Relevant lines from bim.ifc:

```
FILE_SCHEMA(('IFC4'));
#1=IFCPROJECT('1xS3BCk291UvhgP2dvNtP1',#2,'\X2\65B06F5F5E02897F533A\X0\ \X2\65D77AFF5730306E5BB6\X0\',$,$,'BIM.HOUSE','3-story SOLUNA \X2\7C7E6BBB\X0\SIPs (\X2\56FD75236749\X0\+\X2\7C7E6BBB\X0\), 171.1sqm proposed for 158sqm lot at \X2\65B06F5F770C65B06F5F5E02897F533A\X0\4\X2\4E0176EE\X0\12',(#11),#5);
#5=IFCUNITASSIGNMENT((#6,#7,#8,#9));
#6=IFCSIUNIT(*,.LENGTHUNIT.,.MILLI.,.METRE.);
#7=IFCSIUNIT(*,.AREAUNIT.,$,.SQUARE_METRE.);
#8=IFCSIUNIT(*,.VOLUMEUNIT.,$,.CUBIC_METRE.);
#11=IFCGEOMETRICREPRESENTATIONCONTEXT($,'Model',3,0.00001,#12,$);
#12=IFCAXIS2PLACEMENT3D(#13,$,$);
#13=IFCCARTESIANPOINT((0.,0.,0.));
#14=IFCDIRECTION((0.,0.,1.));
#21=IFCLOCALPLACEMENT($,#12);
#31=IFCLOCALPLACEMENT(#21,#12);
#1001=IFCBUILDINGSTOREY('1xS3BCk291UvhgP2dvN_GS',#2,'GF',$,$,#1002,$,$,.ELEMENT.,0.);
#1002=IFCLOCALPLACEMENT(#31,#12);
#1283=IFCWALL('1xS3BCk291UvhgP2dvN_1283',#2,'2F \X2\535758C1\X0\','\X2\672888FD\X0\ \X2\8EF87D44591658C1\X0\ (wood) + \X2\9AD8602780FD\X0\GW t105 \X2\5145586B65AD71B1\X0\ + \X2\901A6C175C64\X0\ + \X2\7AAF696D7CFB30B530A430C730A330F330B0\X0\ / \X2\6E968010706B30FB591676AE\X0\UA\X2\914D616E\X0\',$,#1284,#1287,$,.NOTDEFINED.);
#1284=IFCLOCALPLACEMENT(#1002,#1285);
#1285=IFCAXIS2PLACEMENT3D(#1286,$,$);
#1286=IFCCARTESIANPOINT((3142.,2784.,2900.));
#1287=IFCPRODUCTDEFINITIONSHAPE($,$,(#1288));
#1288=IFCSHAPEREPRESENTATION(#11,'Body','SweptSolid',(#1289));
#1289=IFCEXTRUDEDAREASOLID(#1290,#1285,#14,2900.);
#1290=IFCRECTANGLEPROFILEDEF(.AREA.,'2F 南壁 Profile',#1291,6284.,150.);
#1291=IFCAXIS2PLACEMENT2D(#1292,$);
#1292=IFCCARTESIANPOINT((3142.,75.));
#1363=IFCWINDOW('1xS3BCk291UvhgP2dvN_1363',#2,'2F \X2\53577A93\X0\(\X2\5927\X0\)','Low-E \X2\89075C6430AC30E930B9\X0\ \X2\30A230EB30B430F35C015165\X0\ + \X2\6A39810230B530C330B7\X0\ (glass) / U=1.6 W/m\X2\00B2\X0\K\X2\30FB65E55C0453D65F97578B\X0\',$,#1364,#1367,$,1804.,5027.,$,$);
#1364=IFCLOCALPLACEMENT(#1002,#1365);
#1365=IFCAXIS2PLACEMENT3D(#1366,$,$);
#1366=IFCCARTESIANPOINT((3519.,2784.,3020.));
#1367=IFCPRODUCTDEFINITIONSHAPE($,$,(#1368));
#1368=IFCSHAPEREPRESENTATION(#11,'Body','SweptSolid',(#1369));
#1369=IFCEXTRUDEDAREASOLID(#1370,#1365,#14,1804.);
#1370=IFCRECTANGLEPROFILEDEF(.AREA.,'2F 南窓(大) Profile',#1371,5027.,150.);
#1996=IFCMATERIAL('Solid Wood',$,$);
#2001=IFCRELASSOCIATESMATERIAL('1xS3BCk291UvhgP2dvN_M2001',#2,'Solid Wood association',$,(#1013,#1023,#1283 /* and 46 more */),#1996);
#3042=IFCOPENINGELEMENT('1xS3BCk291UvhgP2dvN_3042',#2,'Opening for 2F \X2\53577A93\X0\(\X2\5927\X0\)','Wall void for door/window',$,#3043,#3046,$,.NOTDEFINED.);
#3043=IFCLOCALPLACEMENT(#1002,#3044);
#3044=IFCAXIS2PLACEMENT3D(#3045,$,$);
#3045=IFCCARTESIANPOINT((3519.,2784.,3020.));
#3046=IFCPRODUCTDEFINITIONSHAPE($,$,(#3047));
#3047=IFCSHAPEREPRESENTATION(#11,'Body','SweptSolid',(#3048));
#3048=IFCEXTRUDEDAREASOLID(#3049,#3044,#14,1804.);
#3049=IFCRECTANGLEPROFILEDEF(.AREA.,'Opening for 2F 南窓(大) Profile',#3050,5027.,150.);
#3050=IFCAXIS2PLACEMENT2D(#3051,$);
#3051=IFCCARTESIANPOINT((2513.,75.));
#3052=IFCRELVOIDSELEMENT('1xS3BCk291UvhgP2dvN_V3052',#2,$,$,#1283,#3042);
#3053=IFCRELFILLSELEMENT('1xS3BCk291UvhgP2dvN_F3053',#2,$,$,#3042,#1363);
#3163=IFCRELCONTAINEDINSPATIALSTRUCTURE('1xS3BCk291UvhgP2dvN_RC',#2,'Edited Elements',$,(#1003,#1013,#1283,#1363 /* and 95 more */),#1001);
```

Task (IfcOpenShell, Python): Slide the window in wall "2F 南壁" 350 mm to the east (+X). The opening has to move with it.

```python
import ifcopenshell
import ifcopenshell.api.geometry
import ifcopenshell.util.placement

model = ifcopenshell.open("bim.ifc")

window = model.by_guid("1xS3BCk291UvhgP2dvN_1363")
opening = window.FillsVoids[0].RelatingOpeningElement
wall = opening.VoidsElements[0].RelatingBuildingElement

wall_matrix = ifcopenshell.util.placement.get_local_placement(wall.ObjectPlacement)
shift = wall_matrix[:3, 0] * 350.0
before = ifcopenshell.util.placement.get_local_placement(window.ObjectPlacement)[:3, 3].copy()

# The window is not placed relative to its opening, so move both.
for product in (opening, window):
    matrix = ifcopenshell.util.placement.get_local_placement(product.ObjectPlacement)
    matrix[:3, 3] += shift
    ifcopenshell.api.geometry.edit_object_placement(model, product=product, matrix=matrix, is_si=False)

after = ifcopenshell.util.placement.get_local_placement(window.ObjectPlacement)[:3, 3]
print("window moved by", (after - before).round(3) + 0.0)

model.write("bim-out.ifc")
```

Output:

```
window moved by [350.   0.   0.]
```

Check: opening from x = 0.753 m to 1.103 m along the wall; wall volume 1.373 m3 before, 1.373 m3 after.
